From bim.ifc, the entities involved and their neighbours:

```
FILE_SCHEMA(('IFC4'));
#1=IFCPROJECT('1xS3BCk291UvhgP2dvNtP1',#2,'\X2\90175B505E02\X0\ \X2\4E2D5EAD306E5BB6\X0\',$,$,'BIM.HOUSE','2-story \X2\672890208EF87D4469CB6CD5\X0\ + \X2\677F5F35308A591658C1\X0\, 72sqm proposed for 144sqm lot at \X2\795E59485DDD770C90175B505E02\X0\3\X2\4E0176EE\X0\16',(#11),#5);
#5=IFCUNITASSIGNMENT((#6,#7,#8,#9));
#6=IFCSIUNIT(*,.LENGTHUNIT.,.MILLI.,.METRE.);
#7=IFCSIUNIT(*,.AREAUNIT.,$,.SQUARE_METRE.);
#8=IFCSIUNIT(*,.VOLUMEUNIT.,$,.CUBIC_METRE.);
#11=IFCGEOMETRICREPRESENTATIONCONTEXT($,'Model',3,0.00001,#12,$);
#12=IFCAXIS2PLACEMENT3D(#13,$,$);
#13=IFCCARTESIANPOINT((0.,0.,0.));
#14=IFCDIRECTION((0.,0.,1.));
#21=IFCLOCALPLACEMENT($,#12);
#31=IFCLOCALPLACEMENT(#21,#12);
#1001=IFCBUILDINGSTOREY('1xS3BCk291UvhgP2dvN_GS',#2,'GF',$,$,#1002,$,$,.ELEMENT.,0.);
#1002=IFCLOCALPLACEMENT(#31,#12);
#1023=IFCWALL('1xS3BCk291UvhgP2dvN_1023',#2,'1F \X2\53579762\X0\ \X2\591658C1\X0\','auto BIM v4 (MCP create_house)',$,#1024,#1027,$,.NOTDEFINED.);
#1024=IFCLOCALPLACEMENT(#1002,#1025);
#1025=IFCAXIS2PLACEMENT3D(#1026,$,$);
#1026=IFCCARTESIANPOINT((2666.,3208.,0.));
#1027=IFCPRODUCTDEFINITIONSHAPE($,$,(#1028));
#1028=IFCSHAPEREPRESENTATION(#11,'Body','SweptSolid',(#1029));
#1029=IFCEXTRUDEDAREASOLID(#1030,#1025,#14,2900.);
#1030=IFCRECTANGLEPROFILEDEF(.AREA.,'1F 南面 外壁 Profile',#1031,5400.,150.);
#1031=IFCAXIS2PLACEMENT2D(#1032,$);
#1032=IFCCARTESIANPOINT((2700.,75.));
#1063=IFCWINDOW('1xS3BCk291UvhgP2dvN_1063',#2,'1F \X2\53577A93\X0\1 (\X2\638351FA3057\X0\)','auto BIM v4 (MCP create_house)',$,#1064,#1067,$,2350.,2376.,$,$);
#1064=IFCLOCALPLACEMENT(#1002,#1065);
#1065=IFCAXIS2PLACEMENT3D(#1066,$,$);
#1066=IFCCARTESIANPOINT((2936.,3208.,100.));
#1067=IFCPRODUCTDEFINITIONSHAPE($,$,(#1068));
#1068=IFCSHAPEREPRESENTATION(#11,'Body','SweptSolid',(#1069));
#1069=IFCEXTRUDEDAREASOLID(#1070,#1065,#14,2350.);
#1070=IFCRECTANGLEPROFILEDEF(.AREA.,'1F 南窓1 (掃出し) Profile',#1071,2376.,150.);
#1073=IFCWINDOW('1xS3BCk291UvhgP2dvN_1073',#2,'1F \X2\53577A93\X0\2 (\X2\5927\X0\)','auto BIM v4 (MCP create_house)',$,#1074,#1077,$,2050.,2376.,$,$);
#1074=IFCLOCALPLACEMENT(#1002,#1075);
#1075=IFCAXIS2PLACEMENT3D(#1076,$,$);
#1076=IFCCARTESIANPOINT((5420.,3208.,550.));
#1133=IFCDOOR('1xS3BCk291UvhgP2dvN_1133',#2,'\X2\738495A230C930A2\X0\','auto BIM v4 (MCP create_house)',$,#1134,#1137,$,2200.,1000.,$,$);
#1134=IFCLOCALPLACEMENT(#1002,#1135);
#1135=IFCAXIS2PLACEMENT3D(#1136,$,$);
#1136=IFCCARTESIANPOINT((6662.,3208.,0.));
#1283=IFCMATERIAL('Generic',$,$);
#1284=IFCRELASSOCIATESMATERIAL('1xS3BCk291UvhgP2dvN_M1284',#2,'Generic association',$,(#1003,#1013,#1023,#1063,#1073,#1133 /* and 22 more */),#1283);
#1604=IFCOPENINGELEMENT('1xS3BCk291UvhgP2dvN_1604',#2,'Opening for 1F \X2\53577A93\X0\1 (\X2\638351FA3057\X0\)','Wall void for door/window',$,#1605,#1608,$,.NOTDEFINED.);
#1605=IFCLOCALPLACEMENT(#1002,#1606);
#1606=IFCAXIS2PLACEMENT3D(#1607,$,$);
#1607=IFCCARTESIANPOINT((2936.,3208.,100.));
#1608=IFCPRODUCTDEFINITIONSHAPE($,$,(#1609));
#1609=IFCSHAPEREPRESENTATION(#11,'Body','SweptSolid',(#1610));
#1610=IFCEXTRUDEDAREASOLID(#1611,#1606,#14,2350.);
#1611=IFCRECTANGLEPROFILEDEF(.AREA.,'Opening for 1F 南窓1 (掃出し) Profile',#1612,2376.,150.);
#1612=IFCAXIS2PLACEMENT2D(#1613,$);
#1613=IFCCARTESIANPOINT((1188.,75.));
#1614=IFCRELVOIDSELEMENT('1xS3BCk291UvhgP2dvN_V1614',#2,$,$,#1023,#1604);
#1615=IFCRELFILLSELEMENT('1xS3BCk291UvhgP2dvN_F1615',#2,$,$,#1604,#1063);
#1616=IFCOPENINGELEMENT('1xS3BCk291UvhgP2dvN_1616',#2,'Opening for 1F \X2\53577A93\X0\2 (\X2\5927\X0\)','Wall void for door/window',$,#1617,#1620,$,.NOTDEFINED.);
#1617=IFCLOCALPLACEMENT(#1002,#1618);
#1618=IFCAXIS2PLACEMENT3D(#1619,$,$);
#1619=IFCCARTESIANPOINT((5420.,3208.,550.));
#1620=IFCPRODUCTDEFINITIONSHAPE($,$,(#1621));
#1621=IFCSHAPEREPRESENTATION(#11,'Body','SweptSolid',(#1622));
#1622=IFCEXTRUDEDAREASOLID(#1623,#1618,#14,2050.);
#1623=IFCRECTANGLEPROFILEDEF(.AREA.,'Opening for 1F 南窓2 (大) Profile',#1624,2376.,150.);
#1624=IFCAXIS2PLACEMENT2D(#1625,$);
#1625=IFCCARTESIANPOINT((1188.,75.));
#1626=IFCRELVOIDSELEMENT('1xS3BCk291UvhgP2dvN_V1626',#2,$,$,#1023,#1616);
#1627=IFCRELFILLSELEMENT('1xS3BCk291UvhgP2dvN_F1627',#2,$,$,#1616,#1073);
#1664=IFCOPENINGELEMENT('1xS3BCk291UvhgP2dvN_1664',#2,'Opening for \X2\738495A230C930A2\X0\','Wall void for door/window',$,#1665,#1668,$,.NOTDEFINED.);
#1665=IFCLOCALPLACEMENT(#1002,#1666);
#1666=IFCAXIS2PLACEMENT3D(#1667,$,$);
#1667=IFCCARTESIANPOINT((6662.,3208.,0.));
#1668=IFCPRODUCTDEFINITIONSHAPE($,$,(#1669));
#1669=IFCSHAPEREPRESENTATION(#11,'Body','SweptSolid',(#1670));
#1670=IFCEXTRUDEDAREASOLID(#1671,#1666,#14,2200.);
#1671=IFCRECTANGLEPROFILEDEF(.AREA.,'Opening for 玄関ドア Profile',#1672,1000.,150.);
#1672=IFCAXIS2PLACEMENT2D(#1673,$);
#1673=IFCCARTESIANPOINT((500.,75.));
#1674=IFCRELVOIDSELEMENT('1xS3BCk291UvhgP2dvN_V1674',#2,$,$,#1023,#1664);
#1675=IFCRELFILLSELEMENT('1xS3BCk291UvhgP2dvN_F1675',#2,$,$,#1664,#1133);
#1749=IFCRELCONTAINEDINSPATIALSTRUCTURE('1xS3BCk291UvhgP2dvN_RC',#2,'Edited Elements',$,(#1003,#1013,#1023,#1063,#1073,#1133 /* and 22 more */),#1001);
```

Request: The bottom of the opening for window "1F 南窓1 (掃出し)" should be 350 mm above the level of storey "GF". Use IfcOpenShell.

```python
import numpy as np
import ifcopenshell
import ifcopenshell.api.geometry
import ifcopenshell.geom
import ifcopenshell.util.element
import ifcopenshell.util.placement
import ifcopenshell.util.shape
import ifcopenshell.util.unit

model = ifcopenshell.open("bim.ifc")
unit_scale = ifcopenshell.util.unit.calculate_unit_scale(model)

window = model.by_guid("1xS3BCk291UvhgP2dvN_1063")
opening = window.FillsVoids[0].RelatingOpeningElement
storey = ifcopenshell.util.element.get_container(window, ifc_class="IfcBuildingStorey")
level = ifcopenshell.util.placement.get_local_placement(storey.ObjectPlacement)[2, 3]

# The opening's origin need not be at the sill, so measure its lowest point.
shape = ifcopenshell.geom.create_shape(ifcopenshell.geom.settings(), opening)
bottom = ifcopenshell.util.shape.get_shape_bottom_elevation(shape, shape.geometry) / unit_scale
dz = level + 350.0 - bottom

shift = np.array([0.0, 0.0, dz])
# The window is not placed relative to its opening, so move both.
for product in (opening, window):
    matrix = ifcopenshell.util.placement.get_local_placement(product.ObjectPlacement)
    matrix[:3, 3] += shift
    ifcopenshell.api.geometry.edit_object_placement(model, product=product, matrix=matrix, is_si=False)

print(f"moved by {dz * unit_scale:+.3f} m")

model.write("bim-out.ifc")
```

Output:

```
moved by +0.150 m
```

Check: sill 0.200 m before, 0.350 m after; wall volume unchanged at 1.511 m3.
